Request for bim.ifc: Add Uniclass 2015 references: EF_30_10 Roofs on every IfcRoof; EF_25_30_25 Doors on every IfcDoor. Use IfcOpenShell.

First a look at what the model holds.

```python
import ifcopenshell

model = ifcopenshell.open("bim.ifc")
print(model.schema)
print("classifications:", [c.Name for c in model.by_type("IfcClassification")])
for ifc_class in ("IfcDoor", "IfcRoof", "IfcStair", "IfcWall", "IfcWindow"):
    print(ifc_class, len(model.by_type(ifc_class)))
```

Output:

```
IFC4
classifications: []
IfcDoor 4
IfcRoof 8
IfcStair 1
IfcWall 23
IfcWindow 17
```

```python
import ifcopenshell
import ifcopenshell.api.classification

model = ifcopenshell.open("bim.ifc")

system = ifcopenshell.api.classification.add_classification(model, classification="Uniclass 2015")

codes = {
    "IfcRoof": ("EF_30_10", "Roofs"),
    "IfcDoor": ("EF_25_30_25", "Doors"),
}
for ifc_class, (code, name) in codes.items():
    products = model.by_type(ifc_class)
    ifcopenshell.api.classification.add_reference(
        model, products=products, classification=system, identification=code, name=name
    )
    print(code, len(products))

model.write("bim_v2.ifc")
```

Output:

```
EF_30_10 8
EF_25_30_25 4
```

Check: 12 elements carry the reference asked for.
